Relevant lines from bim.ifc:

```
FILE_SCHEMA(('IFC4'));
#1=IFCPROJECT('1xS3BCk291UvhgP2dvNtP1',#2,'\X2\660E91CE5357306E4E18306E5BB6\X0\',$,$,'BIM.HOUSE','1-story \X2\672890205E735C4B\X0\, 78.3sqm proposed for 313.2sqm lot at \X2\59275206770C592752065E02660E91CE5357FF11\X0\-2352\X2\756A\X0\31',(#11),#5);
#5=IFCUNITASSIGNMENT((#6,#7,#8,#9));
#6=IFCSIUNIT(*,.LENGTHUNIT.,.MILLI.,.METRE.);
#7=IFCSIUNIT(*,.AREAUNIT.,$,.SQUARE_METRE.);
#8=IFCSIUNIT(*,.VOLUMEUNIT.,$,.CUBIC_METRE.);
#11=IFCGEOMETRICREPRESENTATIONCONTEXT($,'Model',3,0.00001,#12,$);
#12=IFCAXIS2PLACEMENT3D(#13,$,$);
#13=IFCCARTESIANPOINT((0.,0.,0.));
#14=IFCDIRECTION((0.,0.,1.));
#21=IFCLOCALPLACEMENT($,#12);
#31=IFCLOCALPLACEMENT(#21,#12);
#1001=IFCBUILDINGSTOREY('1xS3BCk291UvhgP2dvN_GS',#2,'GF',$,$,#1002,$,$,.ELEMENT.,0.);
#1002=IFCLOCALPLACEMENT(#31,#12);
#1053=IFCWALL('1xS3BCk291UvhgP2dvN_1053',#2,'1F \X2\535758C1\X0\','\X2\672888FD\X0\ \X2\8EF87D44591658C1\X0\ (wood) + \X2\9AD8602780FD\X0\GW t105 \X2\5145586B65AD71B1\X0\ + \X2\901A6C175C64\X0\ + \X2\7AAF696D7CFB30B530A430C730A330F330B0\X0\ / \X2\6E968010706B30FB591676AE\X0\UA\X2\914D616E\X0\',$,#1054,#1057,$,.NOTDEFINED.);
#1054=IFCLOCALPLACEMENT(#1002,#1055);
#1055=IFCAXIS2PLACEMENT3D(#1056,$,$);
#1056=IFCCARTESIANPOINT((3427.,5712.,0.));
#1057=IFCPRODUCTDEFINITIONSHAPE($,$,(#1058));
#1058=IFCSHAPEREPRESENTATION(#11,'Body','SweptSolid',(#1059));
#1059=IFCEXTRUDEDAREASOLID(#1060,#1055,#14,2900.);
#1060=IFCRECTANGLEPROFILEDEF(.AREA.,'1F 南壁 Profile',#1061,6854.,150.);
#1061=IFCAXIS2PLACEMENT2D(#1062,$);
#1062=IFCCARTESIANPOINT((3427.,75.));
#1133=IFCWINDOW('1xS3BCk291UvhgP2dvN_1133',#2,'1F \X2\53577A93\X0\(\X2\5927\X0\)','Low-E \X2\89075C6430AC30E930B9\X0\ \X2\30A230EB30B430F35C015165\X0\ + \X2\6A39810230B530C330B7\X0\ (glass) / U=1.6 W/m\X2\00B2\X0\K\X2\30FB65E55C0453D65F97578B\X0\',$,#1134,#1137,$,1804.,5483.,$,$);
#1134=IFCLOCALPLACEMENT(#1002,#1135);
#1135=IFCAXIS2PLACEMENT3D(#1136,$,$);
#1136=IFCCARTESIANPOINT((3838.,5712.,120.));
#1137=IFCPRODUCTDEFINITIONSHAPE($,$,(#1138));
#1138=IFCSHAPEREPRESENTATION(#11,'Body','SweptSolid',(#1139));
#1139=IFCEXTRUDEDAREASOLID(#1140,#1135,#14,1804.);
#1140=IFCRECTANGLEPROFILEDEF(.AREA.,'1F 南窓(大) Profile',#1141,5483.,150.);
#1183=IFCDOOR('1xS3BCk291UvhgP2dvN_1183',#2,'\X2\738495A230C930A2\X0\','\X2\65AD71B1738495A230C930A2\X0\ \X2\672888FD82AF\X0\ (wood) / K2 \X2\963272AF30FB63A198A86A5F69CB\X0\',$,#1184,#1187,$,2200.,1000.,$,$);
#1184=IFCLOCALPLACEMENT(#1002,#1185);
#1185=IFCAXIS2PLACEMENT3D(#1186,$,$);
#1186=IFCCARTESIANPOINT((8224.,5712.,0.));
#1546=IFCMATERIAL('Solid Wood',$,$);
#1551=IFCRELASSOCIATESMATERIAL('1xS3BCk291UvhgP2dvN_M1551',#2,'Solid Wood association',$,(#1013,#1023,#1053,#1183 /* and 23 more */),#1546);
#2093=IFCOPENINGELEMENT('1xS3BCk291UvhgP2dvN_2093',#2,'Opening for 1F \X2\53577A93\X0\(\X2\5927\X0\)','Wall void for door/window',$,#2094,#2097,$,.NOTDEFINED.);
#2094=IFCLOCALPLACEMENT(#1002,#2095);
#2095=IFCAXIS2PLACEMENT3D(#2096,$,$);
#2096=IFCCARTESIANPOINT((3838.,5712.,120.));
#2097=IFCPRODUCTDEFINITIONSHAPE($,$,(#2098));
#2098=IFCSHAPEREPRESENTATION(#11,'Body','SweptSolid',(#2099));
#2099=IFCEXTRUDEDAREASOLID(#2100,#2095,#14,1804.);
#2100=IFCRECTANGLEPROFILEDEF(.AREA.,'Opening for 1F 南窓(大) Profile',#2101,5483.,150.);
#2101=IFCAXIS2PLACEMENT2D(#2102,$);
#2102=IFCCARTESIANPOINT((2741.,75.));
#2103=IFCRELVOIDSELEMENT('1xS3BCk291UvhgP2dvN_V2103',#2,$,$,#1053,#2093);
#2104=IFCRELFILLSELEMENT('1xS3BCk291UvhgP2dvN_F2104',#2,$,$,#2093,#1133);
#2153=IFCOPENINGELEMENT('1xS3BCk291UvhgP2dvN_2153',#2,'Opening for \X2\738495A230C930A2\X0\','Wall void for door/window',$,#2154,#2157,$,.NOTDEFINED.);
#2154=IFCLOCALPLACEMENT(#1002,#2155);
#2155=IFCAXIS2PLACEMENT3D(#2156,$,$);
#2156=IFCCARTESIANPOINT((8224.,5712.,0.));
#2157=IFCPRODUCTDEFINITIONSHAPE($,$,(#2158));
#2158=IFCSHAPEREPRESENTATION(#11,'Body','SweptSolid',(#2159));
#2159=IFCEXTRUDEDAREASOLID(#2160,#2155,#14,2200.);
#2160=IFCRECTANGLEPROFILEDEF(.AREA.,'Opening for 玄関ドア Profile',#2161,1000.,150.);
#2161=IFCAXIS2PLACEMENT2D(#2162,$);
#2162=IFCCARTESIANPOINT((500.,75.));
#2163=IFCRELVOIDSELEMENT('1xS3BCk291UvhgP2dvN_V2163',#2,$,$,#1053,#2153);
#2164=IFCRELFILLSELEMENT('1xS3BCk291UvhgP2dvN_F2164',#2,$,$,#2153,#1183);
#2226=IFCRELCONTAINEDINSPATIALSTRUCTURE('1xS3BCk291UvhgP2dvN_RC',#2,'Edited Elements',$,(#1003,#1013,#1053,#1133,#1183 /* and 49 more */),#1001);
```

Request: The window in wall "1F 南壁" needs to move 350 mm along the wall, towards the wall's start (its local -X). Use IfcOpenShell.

```python
import ifcopenshell
import ifcopenshell.api.geometry
import ifcopenshell.util.placement
import ifcopenshell.util.unit

model = ifcopenshell.open("bim.ifc")
unit_scale = ifcopenshell.util.unit.calculate_unit_scale(model)

window = model.by_guid("1xS3BCk291UvhgP2dvN_1133")
opening = window.FillsVoids[0].RelatingOpeningElement
wall = opening.VoidsElements[0].RelatingBuildingElement

wall_matrix = ifcopenshell.util.placement.get_local_placement(wall.ObjectPlacement)
shift = wall_matrix[:3, 0] * -0.35 / unit_scale
before = ifcopenshell.util.placement.get_local_placement(window.ObjectPlacement)[:3, 3].copy()

# The window is not placed relative to its opening, so move both.
for product in (opening, window):
    matrix = ifcopenshell.util.placement.get_local_placement(product.ObjectPlacement)
    matrix[:3, 3] += shift
    ifcopenshell.api.geometry.edit_object_placement(model, product=product, matrix=matrix, is_si=False)

after = ifcopenshell.util.placement.get_local_placement(window.ObjectPlacement)[:3, 3]
print("window moved by", (after - before).round(3) + 0.0)

model.write("bim_edited.ifc")
```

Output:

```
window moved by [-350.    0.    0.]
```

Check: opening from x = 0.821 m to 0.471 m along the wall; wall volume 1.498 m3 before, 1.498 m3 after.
